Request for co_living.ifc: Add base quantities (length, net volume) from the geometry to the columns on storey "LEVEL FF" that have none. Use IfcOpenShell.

First a look at what the model holds.

```python
import ifcopenshell
import ifcopenshell.util.element
import ifcopenshell.util.unit

model = ifcopenshell.open("co_living.ifc")
print(model.schema)
for unit_type in ("LENGTHUNIT", "AREAUNIT", "VOLUMEUNIT"):
    print(unit_type, ifcopenshell.util.unit.calculate_unit_scale(model, unit_type))
storey = next(s for s in model.by_type("IfcBuildingStorey") if s.Name == "LEVEL FF")
columns = [e for e in ifcopenshell.util.element.get_decomposition(storey) if e.is_a("IfcColumn")]
for e in sorted(columns, key=lambda e: e.id()):
    print(e.id(), e.is_a(), e.Name, list(ifcopenshell.util.element.get_psets(e, qtos_only=True)), sep=" | ")
```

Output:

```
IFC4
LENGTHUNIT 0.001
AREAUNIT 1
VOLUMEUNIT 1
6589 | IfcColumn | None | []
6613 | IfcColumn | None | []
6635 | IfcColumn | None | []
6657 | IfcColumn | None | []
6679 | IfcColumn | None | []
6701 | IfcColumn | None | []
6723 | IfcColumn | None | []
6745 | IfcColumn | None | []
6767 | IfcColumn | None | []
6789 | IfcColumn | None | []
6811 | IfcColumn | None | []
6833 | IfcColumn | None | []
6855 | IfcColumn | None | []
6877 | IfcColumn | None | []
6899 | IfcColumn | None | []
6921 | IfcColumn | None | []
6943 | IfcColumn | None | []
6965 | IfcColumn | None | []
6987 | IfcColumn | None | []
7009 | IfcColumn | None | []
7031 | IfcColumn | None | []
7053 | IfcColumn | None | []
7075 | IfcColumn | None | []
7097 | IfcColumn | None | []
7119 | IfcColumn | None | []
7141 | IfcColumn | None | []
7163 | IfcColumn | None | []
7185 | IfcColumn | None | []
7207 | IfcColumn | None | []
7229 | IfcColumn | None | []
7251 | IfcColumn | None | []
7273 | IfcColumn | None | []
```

```python
import ifcopenshell
import ifcopenshell.api.pset
import ifcopenshell.geom
import ifcopenshell.util.element
import ifcopenshell.util.shape
import ifcopenshell.util.unit

model = ifcopenshell.open("co_living.ifc")
unit_scale = ifcopenshell.util.unit.calculate_unit_scale(model)
volume_scale = ifcopenshell.util.unit.calculate_unit_scale(model, "VOLUMEUNIT")
settings = ifcopenshell.geom.settings()

storey = next(s for s in model.by_type("IfcBuildingStorey") if s.Name == "LEVEL FF")
columns = [e for e in ifcopenshell.util.element.get_decomposition(storey) if e.is_a("IfcColumn")]

for e in sorted(columns, key=lambda e: e.id()):
    if ifcopenshell.util.element.get_psets(e, qtos_only=True, should_inherit=False):
        continue
    # Geometry comes back in metres, in the element's own axes.
    shape = ifcopenshell.geom.create_shape(settings, e)
    values = {
        "Length": ifcopenshell.util.shape.get_z(shape.geometry) / unit_scale,
        "NetVolume": ifcopenshell.util.shape.get_volume(shape.geometry) / volume_scale,
    }
    qto = ifcopenshell.api.pset.add_qto(model, product=e, name="Qto_ColumnBaseQuantities")
    ifcopenshell.api.pset.edit_qto(model, qto=qto, properties=values)
    print(e.id(), {k: round(v, 3) for k, v in values.items()})

model.write("co_living-out.ifc")
```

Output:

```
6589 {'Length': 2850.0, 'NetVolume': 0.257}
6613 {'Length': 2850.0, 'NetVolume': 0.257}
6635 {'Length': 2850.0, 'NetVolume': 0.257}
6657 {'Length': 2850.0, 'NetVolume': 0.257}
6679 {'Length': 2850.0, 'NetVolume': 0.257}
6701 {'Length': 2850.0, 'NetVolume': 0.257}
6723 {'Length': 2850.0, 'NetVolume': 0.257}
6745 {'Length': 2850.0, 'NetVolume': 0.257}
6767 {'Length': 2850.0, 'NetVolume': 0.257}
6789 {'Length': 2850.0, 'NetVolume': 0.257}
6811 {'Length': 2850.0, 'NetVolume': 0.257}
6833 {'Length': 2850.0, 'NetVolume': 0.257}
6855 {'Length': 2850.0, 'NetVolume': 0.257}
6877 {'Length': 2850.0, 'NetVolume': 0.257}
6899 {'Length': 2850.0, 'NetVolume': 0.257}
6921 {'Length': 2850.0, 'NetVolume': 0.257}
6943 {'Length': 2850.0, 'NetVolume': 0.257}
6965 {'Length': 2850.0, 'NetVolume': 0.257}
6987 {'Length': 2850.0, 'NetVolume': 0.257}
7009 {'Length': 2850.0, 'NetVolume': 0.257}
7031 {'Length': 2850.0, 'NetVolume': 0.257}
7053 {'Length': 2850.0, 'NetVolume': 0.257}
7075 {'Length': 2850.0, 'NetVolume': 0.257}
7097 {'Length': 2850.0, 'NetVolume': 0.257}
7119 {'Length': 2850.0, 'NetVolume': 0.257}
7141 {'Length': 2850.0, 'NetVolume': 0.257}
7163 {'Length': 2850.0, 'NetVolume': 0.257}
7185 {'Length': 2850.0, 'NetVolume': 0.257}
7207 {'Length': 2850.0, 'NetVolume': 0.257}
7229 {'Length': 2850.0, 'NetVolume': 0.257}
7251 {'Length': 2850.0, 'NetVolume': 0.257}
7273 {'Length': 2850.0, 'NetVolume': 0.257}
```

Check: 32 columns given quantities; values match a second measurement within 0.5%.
